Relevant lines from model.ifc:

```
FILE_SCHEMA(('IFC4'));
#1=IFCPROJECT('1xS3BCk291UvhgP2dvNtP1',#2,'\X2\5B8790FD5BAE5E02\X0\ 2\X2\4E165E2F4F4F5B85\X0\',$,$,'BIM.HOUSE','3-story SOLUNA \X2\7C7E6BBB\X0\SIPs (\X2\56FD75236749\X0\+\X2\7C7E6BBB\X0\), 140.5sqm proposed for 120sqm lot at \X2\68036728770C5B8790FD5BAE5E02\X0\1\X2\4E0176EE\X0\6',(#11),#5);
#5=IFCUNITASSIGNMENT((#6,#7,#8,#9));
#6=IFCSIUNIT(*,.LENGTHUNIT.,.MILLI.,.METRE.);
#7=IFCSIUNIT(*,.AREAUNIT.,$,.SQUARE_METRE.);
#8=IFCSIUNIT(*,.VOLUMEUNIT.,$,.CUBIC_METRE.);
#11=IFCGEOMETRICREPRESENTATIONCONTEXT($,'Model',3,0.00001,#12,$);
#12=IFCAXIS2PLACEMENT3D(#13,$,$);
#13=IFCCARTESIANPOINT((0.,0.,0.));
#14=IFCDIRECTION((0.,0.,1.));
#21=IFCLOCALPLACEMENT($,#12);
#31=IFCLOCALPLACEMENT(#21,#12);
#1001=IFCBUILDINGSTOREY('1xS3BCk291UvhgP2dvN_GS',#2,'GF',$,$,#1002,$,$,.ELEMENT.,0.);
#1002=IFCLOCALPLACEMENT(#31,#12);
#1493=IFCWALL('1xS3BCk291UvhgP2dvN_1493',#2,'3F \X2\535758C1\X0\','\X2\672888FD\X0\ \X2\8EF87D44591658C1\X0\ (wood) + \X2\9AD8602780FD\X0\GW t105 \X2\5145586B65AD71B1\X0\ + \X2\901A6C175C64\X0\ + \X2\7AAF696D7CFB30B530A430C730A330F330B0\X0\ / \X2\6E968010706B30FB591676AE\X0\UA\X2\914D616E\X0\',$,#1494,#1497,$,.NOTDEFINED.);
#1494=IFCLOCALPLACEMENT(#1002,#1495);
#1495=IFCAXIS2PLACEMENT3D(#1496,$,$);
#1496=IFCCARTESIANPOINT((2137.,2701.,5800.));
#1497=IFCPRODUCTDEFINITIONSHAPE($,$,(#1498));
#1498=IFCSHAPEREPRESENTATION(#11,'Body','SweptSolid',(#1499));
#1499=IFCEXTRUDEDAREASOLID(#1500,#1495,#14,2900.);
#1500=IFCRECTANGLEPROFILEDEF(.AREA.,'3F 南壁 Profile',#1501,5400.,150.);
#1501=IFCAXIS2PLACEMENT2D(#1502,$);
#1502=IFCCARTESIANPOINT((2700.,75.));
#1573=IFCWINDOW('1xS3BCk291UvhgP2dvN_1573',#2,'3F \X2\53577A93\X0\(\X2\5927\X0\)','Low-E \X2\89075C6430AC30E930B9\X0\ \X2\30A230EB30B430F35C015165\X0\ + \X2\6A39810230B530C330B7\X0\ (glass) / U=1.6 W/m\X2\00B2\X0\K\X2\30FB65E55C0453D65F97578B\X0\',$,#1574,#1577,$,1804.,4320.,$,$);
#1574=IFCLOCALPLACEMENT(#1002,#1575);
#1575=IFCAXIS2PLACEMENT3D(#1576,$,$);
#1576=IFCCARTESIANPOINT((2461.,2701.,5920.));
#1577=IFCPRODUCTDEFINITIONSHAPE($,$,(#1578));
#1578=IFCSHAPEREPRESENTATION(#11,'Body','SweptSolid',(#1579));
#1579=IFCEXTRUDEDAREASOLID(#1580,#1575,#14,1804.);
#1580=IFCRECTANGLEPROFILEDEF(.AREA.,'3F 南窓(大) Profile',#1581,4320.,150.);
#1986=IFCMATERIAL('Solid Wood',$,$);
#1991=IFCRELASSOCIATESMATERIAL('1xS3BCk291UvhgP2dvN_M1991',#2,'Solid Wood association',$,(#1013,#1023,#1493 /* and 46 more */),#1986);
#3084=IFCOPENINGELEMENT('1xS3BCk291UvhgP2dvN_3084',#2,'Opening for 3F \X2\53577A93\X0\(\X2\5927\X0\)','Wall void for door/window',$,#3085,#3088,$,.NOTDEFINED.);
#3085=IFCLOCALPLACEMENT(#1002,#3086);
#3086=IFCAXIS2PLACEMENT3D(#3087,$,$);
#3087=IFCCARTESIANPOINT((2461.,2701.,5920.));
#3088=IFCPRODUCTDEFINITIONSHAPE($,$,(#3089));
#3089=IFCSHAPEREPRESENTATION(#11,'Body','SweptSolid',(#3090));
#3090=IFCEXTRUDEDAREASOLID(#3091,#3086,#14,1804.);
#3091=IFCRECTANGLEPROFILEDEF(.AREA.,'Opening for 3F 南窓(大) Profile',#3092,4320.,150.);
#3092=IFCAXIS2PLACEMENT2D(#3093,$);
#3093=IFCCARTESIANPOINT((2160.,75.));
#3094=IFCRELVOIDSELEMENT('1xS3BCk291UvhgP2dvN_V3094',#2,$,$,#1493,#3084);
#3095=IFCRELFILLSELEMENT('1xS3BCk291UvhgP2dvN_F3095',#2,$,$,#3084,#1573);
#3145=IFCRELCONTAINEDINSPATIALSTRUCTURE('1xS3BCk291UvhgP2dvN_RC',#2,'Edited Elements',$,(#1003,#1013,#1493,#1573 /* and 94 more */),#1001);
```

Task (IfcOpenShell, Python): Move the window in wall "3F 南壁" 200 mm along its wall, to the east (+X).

```python
import ifcopenshell
import ifcopenshell.api.geometry
import ifcopenshell.util.placement
import ifcopenshell.util.unit

model = ifcopenshell.open("model.ifc")
unit_scale = ifcopenshell.util.unit.calculate_unit_scale(model)

window = model.by_guid("1xS3BCk291UvhgP2dvN_1573")
opening = window.FillsVoids[0].RelatingOpeningElement
wall = opening.VoidsElements[0].RelatingBuildingElement

wall_matrix = ifcopenshell.util.placement.get_local_placement(wall.ObjectPlacement)
shift = wall_matrix[:3, 0] * 0.2 / unit_scale
before = ifcopenshell.util.placement.get_local_placement(window.ObjectPlacement)[:3, 3].copy()

# The window is not placed relative to its opening, so move both.
for product in (opening, window):
    matrix = ifcopenshell.util.placement.get_local_placement(product.ObjectPlacement)
    matrix[:3, 3] += shift
    ifcopenshell.api.geometry.edit_object_placement(model, product=product, matrix=matrix, is_si=False)

after = ifcopenshell.util.placement.get_local_placement(window.ObjectPlacement)[:3, 3]
print("window moved by", (after - before).round(3) + 0.0)

model.write("model_rev.ifc")
```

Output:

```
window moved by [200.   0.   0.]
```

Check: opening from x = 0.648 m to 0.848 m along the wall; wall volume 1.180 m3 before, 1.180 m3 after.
